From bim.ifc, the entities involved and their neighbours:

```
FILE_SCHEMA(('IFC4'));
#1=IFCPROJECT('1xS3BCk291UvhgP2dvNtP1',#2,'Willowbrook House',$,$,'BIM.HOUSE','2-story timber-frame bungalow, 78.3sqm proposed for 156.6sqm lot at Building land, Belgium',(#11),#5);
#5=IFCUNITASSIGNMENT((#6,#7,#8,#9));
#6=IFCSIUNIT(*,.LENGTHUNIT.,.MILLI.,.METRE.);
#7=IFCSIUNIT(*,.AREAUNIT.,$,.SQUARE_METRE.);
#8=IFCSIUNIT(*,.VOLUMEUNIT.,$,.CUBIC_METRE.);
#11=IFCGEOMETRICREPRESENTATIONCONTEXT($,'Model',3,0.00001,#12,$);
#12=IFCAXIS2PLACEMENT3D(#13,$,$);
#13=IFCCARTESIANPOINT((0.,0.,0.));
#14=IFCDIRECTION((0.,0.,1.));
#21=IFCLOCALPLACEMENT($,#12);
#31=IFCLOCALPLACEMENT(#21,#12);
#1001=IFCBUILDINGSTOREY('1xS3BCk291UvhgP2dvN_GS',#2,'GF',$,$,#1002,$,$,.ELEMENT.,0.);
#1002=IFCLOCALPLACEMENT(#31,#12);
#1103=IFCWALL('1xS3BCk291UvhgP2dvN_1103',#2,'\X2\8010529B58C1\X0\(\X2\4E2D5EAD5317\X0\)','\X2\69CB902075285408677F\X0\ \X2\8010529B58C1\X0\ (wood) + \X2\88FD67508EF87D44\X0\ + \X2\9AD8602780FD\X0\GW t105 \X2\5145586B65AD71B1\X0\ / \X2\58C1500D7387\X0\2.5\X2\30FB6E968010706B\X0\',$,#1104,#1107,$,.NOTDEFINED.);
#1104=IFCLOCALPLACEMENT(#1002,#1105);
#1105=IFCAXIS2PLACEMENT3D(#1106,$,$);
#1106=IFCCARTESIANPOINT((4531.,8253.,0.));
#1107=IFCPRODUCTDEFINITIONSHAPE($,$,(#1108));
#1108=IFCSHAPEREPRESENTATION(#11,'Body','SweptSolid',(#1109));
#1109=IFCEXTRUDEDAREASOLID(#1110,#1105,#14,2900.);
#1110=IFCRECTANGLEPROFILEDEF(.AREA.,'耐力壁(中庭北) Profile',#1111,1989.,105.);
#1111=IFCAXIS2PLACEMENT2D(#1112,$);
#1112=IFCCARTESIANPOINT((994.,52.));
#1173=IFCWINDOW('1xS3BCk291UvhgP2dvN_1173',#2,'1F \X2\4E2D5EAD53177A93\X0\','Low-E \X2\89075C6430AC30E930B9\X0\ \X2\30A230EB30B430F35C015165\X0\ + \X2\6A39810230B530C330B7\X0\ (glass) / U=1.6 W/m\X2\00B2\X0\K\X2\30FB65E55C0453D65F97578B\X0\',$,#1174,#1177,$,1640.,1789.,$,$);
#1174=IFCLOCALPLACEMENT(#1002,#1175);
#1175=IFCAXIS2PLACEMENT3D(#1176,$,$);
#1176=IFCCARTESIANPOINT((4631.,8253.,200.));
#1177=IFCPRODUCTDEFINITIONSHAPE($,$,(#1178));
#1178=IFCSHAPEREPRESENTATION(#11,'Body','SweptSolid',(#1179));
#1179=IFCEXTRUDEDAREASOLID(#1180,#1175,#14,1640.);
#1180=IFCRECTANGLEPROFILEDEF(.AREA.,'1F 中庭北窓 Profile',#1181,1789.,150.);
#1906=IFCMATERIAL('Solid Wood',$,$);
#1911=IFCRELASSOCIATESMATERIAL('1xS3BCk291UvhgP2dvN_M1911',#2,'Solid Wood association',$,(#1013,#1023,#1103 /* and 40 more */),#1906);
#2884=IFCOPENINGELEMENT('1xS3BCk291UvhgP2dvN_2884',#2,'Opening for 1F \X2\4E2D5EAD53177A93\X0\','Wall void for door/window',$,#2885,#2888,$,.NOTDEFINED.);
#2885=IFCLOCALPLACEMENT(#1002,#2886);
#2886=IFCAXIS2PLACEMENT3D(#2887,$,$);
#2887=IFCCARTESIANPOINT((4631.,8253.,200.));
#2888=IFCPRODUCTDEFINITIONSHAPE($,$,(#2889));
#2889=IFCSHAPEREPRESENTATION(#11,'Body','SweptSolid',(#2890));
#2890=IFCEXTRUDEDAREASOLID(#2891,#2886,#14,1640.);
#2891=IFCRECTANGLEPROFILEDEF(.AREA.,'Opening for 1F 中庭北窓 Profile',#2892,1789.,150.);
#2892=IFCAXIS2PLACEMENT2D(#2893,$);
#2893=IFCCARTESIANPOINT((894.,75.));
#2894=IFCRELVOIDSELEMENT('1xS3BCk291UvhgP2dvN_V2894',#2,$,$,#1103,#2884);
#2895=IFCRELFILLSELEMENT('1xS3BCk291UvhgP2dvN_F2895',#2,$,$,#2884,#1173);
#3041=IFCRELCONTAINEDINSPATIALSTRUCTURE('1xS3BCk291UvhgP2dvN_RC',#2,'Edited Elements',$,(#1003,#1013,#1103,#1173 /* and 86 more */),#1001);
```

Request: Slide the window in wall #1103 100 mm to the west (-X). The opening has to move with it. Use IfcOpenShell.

```python
import ifcopenshell
import ifcopenshell.api.geometry
import ifcopenshell.util.placement

model = ifcopenshell.open("bim.ifc")

window = model.by_guid("1xS3BCk291UvhgP2dvN_1173")
opening = window.FillsVoids[0].RelatingOpeningElement
wall = opening.VoidsElements[0].RelatingBuildingElement

wall_matrix = ifcopenshell.util.placement.get_local_placement(wall.ObjectPlacement)
shift = wall_matrix[:3, 0] * -100.0
before = ifcopenshell.util.placement.get_local_placement(window.ObjectPlacement)[:3, 3].copy()

# The window is not placed relative to its opening, so move both.
for product in (opening, window):
    matrix = ifcopenshell.util.placement.get_local_placement(product.ObjectPlacement)
    matrix[:3, 3] += shift
    ifcopenshell.api.geometry.edit_object_placement(model, product=product, matrix=matrix, is_si=False)

after = ifcopenshell.util.placement.get_local_placement(window.ObjectPlacement)[:3, 3]
print("window moved by", (after - before).round(3) + 0.0)

model.write("bim-out.ifc")
```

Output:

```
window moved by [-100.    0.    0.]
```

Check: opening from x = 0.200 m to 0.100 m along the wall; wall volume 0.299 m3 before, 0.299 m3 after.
